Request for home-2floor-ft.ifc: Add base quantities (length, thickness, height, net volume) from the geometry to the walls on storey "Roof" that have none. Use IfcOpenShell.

First a look at what the model holds.

```python
import ifcopenshell
import ifcopenshell.util.element
import ifcopenshell.util.unit

model = ifcopenshell.open("home-2floor-ft.ifc")
print(model.schema)
for unit_type in ("LENGTHUNIT", "AREAUNIT", "VOLUMEUNIT"):
    print(unit_type, ifcopenshell.util.unit.calculate_unit_scale(model, unit_type))
storey = next(s for s in model.by_type("IfcBuildingStorey") if s.Name == "Roof")
walls = [e for e in ifcopenshell.util.element.get_decomposition(storey) if e.is_a("IfcWall")]
for e in sorted(walls, key=lambda e: e.id()):
    print(e.id(), e.is_a(), e.Name, list(ifcopenshell.util.element.get_psets(e, qtos_only=True)), sep=" | ")
```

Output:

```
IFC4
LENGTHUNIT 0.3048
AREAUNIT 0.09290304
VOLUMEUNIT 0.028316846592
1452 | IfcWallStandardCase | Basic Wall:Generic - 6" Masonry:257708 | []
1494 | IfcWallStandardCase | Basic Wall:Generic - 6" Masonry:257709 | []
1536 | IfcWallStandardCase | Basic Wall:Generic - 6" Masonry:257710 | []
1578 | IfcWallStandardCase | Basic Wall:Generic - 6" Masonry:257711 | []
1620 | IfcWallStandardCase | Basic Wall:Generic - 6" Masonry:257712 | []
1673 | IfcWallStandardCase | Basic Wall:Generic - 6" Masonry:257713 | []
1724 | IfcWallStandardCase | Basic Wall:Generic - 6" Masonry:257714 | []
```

```python
import ifcopenshell
import ifcopenshell.api.pset
import ifcopenshell.geom
import ifcopenshell.util.element
import ifcopenshell.util.shape
import ifcopenshell.util.unit

model = ifcopenshell.open("home-2floor-ft.ifc")
unit_scale = ifcopenshell.util.unit.calculate_unit_scale(model)
volume_scale = ifcopenshell.util.unit.calculate_unit_scale(model, "VOLUMEUNIT")
settings = ifcopenshell.geom.settings()

storey = next(s for s in model.by_type("IfcBuildingStorey") if s.Name == "Roof")
walls = [e for e in ifcopenshell.util.element.get_decomposition(storey) if e.is_a("IfcWall")]

for e in sorted(walls, key=lambda e: e.id()):
    if ifcopenshell.util.element.get_psets(e, qtos_only=True, should_inherit=False):
        continue
    # Geometry comes back in metres, in the element's own axes.
    shape = ifcopenshell.geom.create_shape(settings, e)
    values = {
        "Length": ifcopenshell.util.shape.get_x(shape.geometry) / unit_scale,
        "Width": ifcopenshell.util.shape.get_y(shape.geometry) / unit_scale,
        "Height": ifcopenshell.util.shape.get_z(shape.geometry) / unit_scale,
        "NetVolume": ifcopenshell.util.shape.get_volume(shape.geometry) / volume_scale,
    }
    qto = ifcopenshell.api.pset.add_qto(model, product=e, name="Qto_WallBaseQuantities")
    ifcopenshell.api.pset.edit_qto(model, qto=qto, properties=values)
    print(e.id(), {k: round(v, 3) for k, v in values.items()})

model.write("home-2floor-ft_updated.ifc")
```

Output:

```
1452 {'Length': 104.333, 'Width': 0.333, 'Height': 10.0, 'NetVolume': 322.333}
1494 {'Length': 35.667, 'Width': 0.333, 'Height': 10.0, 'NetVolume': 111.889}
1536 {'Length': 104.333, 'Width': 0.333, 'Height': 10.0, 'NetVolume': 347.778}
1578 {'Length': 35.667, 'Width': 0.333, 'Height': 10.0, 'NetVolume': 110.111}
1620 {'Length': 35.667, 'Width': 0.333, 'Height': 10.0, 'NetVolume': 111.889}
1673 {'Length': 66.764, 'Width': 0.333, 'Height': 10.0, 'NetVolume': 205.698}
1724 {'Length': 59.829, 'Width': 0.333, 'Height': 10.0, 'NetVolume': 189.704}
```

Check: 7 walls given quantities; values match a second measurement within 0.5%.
